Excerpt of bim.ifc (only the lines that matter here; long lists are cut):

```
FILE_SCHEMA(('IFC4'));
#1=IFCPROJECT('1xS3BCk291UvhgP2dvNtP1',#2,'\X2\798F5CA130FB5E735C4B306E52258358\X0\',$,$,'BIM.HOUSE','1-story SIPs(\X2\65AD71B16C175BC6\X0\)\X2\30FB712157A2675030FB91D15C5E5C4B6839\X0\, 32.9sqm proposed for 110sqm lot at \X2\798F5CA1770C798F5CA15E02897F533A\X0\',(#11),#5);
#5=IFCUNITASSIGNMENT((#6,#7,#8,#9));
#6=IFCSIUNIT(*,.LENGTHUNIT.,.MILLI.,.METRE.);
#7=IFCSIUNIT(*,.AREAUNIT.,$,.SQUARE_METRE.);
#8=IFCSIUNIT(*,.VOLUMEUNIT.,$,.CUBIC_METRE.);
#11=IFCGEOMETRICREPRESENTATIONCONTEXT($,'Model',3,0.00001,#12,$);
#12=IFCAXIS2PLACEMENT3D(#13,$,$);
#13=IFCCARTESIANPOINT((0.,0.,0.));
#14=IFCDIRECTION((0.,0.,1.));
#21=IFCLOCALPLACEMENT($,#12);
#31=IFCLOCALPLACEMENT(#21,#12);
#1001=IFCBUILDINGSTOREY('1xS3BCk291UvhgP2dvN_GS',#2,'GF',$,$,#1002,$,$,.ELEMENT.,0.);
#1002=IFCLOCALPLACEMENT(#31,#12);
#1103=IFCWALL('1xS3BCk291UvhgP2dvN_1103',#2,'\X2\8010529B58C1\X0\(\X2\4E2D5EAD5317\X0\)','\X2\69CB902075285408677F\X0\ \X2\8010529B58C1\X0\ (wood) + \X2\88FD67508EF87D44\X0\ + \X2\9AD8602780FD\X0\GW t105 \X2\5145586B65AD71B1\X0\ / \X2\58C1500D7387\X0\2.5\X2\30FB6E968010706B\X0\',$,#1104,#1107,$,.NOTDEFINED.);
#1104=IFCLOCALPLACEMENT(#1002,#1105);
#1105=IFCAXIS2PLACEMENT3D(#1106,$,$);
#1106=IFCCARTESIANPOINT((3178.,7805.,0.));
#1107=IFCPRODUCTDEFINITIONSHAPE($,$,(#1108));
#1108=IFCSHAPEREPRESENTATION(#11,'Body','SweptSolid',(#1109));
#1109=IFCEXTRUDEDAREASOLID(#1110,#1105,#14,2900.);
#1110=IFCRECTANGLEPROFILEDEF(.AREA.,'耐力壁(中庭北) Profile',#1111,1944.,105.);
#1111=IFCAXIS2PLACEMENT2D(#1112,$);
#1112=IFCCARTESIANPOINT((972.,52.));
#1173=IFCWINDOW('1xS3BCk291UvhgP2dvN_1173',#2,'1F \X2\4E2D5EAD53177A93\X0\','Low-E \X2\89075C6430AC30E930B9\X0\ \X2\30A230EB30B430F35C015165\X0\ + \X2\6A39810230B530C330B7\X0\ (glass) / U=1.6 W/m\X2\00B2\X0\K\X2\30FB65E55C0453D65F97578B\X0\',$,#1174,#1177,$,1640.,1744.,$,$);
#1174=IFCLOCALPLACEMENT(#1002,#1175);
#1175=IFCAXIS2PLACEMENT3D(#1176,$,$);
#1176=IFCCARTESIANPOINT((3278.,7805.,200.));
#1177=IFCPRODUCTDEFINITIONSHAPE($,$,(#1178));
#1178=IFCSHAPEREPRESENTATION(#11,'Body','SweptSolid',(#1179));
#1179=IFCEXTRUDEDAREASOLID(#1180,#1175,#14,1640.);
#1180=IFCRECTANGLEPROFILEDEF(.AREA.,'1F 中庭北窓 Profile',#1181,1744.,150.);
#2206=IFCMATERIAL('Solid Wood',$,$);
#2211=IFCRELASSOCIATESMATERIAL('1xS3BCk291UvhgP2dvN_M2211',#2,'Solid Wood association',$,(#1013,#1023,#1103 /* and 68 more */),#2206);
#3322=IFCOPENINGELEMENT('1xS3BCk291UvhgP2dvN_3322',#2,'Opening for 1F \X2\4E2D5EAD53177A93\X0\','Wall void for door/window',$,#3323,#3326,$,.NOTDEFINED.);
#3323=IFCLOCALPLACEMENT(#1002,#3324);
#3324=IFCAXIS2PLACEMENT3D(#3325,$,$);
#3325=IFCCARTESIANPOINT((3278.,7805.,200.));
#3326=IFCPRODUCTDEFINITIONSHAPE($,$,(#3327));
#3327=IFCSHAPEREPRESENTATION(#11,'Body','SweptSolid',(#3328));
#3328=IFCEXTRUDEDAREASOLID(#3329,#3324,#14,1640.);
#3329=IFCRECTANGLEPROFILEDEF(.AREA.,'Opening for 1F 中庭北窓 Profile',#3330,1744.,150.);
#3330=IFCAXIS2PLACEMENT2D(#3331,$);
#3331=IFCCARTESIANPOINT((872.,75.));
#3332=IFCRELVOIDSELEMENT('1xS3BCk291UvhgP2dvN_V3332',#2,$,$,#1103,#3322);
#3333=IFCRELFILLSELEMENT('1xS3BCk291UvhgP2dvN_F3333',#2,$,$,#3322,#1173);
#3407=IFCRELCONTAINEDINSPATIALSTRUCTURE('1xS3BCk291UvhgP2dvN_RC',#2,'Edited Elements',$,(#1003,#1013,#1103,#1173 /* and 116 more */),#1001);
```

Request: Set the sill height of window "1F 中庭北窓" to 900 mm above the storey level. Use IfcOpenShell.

```python
import numpy as np
import ifcopenshell
import ifcopenshell.api.geometry
import ifcopenshell.geom
import ifcopenshell.util.element
import ifcopenshell.util.placement
import ifcopenshell.util.shape
import ifcopenshell.util.unit

model = ifcopenshell.open("bim.ifc")
unit_scale = ifcopenshell.util.unit.calculate_unit_scale(model)

window = model.by_guid("1xS3BCk291UvhgP2dvN_1173")
opening = window.FillsVoids[0].RelatingOpeningElement
storey = ifcopenshell.util.element.get_container(window, ifc_class="IfcBuildingStorey")
level = ifcopenshell.util.placement.get_local_placement(storey.ObjectPlacement)[2, 3]

# The opening's origin need not be at the sill, so measure its lowest point.
shape = ifcopenshell.geom.create_shape(ifcopenshell.geom.settings(), opening)
bottom = ifcopenshell.util.shape.get_shape_bottom_elevation(shape, shape.geometry) / unit_scale
dz = level + 0.9 / unit_scale - bottom

shift = np.array([0.0, 0.0, dz])
# The window is not placed relative to its opening, so move both.
for product in (opening, window):
    matrix = ifcopenshell.util.placement.get_local_placement(product.ObjectPlacement)
    matrix[:3, 3] += shift
    ifcopenshell.api.geometry.edit_object_placement(model, product=product, matrix=matrix, is_si=False)

print(f"moved by {dz * unit_scale:+.3f} m")

model.write("bim_v2.ifc")
```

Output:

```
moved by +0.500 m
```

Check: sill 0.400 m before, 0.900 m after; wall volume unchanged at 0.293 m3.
